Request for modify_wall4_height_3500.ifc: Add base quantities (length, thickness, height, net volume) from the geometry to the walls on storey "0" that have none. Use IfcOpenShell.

First a look at what the model holds.

```python
import ifcopenshell
import ifcopenshell.util.element
import ifcopenshell.util.unit

model = ifcopenshell.open("modify_wall4_height_3500.ifc")
print(model.schema)
for unit_type in ("LENGTHUNIT", "AREAUNIT", "VOLUMEUNIT"):
    print(unit_type, ifcopenshell.util.unit.calculate_unit_scale(model, unit_type))
storey = next(s for s in model.by_type("IfcBuildingStorey") if s.Name == "0")
walls = [e for e in ifcopenshell.util.element.get_decomposition(storey) if e.is_a("IfcWall")]
for e in sorted(walls, key=lambda e: e.id()):
    print(e.id(), e.is_a(), e.Name, list(ifcopenshell.util.element.get_psets(e, qtos_only=True)), sep=" | ")
```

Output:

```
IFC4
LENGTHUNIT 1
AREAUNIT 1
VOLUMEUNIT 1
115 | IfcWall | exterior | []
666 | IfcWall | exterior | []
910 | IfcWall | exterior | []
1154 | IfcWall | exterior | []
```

```python
import ifcopenshell
import ifcopenshell.api.pset
import ifcopenshell.geom
import ifcopenshell.util.element
import ifcopenshell.util.shape
import ifcopenshell.util.unit

model = ifcopenshell.open("modify_wall4_height_3500.ifc")
unit_scale = ifcopenshell.util.unit.calculate_unit_scale(model)
volume_scale = ifcopenshell.util.unit.calculate_unit_scale(model, "VOLUMEUNIT")
settings = ifcopenshell.geom.settings()

storey = next(s for s in model.by_type("IfcBuildingStorey") if s.Name == "0")
walls = [e for e in ifcopenshell.util.element.get_decomposition(storey) if e.is_a("IfcWall")]

for e in sorted(walls, key=lambda e: e.id()):
    if ifcopenshell.util.element.get_psets(e, qtos_only=True, should_inherit=False):
        continue
    # Geometry comes back in metres, in the element's own axes.
    shape = ifcopenshell.geom.create_shape(settings, e)
    values = {
        "Length": ifcopenshell.util.shape.get_x(shape.geometry) / unit_scale,
        "Width": ifcopenshell.util.shape.get_y(shape.geometry) / unit_scale,
        "Height": ifcopenshell.util.shape.get_z(shape.geometry) / unit_scale,
        "NetVolume": ifcopenshell.util.shape.get_volume(shape.geometry) / volume_scale,
    }
    qto = ifcopenshell.api.pset.add_qto(model, product=e, name="Qto_WallBaseQuantities")
    ifcopenshell.api.pset.edit_qto(model, qto=qto, properties=values)
    print(e.id(), {k: round(v, 3) for k, v in values.items()})

model.write("modify_wall4_height_3500_rev.ifc")
```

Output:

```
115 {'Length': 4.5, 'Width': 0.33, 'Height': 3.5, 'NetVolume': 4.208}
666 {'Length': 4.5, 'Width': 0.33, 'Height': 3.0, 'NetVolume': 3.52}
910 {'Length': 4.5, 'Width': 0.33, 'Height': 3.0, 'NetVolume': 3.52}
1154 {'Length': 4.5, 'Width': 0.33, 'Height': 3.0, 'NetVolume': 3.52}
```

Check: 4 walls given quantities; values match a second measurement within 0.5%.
